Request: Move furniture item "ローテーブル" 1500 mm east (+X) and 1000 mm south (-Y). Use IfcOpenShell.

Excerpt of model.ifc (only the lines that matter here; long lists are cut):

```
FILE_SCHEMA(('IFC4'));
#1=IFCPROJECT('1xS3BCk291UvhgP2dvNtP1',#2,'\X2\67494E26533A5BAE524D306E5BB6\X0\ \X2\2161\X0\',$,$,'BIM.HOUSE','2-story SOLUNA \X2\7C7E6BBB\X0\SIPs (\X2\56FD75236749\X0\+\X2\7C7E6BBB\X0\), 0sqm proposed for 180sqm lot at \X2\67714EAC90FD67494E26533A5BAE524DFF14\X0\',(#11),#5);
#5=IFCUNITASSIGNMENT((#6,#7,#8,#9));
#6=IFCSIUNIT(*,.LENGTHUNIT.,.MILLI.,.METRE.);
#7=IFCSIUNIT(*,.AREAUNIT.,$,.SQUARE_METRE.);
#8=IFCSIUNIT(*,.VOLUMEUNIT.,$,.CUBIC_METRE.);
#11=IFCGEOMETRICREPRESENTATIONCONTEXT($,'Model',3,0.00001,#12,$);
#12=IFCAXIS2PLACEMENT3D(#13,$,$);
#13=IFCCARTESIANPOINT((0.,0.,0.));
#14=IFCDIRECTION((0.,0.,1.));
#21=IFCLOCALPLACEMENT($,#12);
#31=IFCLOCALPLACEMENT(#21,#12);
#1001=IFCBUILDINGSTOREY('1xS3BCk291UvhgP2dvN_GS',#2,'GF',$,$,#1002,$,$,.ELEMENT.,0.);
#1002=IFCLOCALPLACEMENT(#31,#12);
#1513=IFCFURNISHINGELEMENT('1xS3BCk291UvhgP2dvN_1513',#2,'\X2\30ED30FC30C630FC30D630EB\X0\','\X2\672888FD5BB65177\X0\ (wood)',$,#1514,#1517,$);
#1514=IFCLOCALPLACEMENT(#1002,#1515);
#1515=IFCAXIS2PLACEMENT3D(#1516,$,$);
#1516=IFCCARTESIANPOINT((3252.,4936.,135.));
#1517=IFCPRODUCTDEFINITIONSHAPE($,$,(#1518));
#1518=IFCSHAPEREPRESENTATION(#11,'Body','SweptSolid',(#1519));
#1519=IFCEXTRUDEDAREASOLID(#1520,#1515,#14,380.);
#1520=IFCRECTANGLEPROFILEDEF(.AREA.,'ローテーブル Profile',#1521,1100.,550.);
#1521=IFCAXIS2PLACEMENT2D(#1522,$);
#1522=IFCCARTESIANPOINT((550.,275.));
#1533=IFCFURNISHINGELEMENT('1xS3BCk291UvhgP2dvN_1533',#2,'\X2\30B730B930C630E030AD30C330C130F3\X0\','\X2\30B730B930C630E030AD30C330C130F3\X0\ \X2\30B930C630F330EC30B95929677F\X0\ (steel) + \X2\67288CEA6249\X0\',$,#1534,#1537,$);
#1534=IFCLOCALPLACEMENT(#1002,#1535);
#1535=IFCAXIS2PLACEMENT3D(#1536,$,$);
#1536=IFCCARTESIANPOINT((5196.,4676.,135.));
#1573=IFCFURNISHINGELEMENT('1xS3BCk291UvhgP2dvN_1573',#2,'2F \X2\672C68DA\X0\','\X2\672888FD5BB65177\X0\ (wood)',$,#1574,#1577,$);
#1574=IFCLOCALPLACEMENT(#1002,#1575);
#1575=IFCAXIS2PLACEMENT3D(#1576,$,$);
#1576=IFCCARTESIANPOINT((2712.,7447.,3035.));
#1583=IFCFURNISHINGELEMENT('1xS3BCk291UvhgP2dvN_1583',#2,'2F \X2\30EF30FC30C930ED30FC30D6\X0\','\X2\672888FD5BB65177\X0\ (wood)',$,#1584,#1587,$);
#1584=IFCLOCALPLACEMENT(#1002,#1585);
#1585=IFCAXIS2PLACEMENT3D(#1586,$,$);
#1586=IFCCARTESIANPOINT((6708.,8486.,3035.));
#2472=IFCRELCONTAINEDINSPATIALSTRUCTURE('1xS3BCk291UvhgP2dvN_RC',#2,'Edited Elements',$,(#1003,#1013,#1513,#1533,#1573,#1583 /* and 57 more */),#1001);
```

```python
import ifcopenshell
import ifcopenshell.api.geometry
import ifcopenshell.util.placement
import ifcopenshell.util.unit

model = ifcopenshell.open("model.ifc")
unit_scale = ifcopenshell.util.unit.calculate_unit_scale(model)

item = model.by_guid("1xS3BCk291UvhgP2dvN_1513")
matrix = ifcopenshell.util.placement.get_local_placement(item.ObjectPlacement)
matrix[0, 3] += 1.5 / unit_scale
matrix[1, 3] -= 1 / unit_scale
ifcopenshell.api.geometry.edit_object_placement(model, product=item, matrix=matrix, is_si=False)

print(ifcopenshell.util.placement.get_local_placement(item.ObjectPlacement).round(3) + 0.0)

model.write("model_rev.ifc")
```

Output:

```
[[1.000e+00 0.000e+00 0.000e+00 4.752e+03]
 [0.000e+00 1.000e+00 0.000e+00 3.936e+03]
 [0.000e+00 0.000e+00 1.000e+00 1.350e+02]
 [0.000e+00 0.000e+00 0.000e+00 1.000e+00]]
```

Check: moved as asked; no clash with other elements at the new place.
